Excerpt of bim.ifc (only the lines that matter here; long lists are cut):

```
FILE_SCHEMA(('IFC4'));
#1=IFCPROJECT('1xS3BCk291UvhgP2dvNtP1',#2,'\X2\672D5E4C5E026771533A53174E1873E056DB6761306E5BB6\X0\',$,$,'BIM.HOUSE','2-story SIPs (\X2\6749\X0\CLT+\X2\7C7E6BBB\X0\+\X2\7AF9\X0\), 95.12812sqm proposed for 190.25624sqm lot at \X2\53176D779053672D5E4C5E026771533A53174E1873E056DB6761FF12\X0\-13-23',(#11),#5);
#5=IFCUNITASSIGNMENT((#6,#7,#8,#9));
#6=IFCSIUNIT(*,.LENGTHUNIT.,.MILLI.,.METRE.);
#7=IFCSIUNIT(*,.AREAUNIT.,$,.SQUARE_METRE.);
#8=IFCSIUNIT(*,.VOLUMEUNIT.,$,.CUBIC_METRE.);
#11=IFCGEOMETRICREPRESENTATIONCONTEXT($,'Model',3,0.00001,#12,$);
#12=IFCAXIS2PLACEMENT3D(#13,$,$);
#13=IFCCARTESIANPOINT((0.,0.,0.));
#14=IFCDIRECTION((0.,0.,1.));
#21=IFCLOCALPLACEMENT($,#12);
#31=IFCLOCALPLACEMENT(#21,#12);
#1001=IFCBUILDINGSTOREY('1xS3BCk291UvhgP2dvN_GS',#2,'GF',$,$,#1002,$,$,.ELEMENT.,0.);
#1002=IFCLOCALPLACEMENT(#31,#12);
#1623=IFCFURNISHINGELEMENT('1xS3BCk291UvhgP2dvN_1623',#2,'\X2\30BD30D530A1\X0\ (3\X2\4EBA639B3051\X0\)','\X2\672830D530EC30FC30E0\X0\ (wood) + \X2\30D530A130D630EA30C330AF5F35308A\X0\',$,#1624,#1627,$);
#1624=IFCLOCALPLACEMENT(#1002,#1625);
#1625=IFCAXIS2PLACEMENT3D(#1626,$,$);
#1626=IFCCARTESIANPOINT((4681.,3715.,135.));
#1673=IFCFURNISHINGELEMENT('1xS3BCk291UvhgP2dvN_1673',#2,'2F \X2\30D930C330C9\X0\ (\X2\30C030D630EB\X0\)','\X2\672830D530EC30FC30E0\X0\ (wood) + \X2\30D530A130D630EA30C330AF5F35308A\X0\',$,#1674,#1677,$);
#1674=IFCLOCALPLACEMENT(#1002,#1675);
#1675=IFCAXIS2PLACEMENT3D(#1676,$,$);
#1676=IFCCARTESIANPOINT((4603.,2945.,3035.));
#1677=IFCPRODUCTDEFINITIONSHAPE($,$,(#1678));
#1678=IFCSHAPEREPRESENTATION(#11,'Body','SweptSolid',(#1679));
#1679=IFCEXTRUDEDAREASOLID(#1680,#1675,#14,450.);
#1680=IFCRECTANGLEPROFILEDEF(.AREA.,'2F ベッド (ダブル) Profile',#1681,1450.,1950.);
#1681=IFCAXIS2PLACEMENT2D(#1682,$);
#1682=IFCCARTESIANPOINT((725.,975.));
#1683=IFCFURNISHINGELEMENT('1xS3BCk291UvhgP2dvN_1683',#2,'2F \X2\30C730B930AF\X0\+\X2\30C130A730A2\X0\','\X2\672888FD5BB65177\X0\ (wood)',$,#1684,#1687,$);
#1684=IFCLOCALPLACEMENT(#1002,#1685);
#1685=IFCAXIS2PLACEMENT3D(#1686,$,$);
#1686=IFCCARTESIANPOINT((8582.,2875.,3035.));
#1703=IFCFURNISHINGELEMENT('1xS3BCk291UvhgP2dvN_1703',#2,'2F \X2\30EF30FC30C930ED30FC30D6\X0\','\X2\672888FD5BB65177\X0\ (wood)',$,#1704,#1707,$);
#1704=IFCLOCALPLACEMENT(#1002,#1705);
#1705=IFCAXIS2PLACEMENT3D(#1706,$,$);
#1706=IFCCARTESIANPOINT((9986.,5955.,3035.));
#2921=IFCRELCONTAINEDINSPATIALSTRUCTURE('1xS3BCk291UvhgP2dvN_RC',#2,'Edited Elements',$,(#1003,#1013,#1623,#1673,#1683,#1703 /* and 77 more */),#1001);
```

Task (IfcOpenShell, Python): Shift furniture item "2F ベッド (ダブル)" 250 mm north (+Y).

```python
import ifcopenshell
import ifcopenshell.api.geometry
import ifcopenshell.util.placement

model = ifcopenshell.open("bim.ifc")

item = model.by_guid("1xS3BCk291UvhgP2dvN_1673")
matrix = ifcopenshell.util.placement.get_local_placement(item.ObjectPlacement)
matrix[1, 3] += 250.0
ifcopenshell.api.geometry.edit_object_placement(model, product=item, matrix=matrix, is_si=False)

print(ifcopenshell.util.placement.get_local_placement(item.ObjectPlacement).round(3) + 0.0)

model.write("bim_edited.ifc")
```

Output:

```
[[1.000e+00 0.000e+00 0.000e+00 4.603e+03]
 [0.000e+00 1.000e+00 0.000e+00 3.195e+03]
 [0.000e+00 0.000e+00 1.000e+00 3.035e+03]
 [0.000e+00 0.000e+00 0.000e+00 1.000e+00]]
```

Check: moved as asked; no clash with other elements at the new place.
